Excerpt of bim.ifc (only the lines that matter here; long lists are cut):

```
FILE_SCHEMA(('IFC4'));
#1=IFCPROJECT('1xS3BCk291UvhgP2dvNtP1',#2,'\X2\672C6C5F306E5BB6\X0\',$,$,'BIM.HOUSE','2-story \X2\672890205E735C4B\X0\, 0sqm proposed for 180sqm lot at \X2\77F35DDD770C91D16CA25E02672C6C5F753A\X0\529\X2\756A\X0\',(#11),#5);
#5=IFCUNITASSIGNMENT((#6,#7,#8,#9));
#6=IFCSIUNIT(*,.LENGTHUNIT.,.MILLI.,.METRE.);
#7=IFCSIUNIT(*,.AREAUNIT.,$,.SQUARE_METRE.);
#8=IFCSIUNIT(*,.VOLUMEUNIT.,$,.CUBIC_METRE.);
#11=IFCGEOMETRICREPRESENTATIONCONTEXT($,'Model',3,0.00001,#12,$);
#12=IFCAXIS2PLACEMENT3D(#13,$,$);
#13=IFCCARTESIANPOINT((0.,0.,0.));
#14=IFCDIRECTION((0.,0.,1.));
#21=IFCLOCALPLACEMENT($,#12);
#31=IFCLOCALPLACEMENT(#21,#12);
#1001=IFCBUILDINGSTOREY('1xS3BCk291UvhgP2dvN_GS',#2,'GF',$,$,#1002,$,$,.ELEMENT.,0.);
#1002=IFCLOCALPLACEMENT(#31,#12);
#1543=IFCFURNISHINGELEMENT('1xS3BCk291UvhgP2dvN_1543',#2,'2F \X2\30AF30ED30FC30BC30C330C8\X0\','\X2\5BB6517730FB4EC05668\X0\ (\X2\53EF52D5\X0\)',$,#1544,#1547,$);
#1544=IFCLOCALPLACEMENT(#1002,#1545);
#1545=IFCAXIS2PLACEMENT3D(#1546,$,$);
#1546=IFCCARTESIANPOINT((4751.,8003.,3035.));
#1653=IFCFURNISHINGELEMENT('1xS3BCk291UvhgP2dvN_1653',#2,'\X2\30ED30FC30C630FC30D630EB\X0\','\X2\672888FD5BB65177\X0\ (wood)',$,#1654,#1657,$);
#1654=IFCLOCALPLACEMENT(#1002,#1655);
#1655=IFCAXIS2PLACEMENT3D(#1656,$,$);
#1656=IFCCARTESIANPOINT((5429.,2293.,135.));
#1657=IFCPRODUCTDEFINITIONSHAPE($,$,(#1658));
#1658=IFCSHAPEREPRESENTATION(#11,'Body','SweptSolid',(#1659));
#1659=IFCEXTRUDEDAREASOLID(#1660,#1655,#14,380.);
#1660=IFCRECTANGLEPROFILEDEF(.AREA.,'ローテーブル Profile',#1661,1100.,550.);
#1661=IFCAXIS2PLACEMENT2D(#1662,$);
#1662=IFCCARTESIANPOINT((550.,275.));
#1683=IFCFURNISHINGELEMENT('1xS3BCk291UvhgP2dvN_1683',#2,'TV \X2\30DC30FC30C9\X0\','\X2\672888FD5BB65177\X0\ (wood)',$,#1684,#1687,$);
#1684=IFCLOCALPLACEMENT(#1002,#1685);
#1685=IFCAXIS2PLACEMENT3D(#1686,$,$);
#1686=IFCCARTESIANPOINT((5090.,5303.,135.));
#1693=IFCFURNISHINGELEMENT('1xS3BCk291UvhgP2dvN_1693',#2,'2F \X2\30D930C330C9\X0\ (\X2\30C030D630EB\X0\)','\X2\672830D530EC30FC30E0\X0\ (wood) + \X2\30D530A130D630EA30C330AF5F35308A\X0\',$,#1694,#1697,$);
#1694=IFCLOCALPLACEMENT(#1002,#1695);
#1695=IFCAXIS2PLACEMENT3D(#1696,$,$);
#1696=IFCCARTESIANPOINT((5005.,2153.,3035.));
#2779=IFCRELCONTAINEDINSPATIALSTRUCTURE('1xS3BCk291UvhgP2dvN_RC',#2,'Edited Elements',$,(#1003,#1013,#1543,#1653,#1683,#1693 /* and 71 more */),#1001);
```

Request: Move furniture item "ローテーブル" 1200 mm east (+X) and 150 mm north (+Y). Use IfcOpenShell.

```python
import ifcopenshell
import ifcopenshell.api.geometry
import ifcopenshell.util.placement

model = ifcopenshell.open("bim.ifc")

item = model.by_id(1653)
matrix = ifcopenshell.util.placement.get_local_placement(item.ObjectPlacement)
matrix[0, 3] += 1200.0
matrix[1, 3] += 150.0
ifcopenshell.api.geometry.edit_object_placement(model, product=item, matrix=matrix, is_si=False)

print(ifcopenshell.util.placement.get_local_placement(item.ObjectPlacement).round(3) + 0.0)

model.write("bim_edited.ifc")
```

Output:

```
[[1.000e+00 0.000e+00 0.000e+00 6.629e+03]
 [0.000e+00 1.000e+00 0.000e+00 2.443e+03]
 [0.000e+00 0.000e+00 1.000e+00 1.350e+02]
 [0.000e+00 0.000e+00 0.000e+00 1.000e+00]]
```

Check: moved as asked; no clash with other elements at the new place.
